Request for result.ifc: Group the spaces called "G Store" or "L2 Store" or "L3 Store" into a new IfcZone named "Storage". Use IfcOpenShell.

First a look at what the model holds.

```python
import ifcopenshell

model = ifcopenshell.open("result.ifc")
print(model.schema)
seen = {}
for space in model.by_type("IfcSpace"):
    seen[space.LongName] = seen.get(space.LongName, 0) + 1
for name, count in sorted(seen.items(), key=str):
    print(count, "x", name)
print("zones:", [z.Name for z in model.by_type("IfcZone")][:20])
```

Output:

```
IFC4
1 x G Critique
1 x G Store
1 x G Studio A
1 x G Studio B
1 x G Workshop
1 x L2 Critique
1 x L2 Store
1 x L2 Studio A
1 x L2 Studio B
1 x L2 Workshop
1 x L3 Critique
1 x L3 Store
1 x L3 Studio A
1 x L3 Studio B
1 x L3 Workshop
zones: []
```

```python
import ifcopenshell
import ifcopenshell.api.group
import ifcopenshell.api.root

model = ifcopenshell.open("result.ifc")

names = {"G Store", "L2 Store", "L3 Store"}
spaces = [s for s in model.by_type("IfcSpace") if s.LongName in names]

zone = ifcopenshell.api.root.create_entity(model, ifc_class="IfcZone", name="Storage")
ifcopenshell.api.group.assign_group(model, products=spaces, group=zone)
print(len(spaces), "spaces in", zone.Name)

model.write("result_v2.ifc")
```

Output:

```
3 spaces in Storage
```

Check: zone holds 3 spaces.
